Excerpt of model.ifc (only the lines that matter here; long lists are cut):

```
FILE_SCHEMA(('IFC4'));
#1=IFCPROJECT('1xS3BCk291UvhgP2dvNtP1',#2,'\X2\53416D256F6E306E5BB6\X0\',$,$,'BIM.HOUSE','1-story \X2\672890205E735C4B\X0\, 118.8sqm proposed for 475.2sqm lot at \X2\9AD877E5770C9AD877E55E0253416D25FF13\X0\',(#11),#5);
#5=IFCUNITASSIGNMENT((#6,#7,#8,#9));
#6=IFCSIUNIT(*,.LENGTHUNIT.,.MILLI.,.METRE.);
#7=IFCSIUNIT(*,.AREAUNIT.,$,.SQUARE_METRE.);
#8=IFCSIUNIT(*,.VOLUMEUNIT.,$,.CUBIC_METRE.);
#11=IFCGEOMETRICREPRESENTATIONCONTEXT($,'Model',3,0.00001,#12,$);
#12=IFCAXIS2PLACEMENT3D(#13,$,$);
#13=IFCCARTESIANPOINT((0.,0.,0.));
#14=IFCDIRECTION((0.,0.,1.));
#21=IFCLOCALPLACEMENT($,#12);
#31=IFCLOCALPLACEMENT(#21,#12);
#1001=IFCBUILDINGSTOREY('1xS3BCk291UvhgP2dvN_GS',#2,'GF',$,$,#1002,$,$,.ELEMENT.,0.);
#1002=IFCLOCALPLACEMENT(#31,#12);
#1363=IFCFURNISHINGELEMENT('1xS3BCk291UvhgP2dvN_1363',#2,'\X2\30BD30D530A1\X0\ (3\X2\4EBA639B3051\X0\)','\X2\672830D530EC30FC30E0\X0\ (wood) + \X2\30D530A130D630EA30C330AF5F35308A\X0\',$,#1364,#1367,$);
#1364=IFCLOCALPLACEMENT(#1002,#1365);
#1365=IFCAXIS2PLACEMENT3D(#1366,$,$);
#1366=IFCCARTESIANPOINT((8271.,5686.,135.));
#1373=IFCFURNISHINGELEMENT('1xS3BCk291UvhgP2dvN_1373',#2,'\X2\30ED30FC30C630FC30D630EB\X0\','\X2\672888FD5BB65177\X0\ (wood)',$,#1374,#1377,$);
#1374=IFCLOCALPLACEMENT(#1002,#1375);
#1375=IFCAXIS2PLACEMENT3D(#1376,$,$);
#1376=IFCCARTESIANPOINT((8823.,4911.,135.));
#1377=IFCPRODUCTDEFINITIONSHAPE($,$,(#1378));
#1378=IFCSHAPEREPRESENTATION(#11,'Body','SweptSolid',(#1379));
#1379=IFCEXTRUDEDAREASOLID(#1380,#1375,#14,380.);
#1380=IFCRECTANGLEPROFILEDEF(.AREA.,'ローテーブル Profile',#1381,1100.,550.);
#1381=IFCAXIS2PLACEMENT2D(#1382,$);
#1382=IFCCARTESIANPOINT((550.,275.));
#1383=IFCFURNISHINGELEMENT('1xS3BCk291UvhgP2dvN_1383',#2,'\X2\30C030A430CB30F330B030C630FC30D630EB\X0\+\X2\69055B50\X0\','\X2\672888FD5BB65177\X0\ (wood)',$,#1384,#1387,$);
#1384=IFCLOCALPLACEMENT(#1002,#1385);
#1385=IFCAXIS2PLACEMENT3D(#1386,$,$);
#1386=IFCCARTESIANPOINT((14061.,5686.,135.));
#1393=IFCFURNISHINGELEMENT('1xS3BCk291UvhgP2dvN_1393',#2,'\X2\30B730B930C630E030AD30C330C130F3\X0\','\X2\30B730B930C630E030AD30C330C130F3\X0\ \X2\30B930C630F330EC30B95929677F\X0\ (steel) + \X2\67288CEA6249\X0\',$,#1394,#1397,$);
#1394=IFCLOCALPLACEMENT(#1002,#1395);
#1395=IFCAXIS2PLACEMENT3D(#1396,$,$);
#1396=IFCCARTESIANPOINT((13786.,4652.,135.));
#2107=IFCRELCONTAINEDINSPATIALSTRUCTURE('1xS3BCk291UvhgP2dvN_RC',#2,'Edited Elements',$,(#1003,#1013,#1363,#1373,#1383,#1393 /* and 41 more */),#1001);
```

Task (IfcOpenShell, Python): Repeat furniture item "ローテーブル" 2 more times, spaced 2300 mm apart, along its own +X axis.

```python
import ifcopenshell
import ifcopenshell.api.geometry
import ifcopenshell.api.root
import ifcopenshell.util.element
import ifcopenshell.util.placement

model = ifcopenshell.open("model.ifc")


def reuse_history(source, copy):
    """copy_class also copies each property set's owner history, people and application; keep the originals."""
    for rel in copy.IsDefinedBy:
        if rel.is_a("IfcRelDefinesByProperties") and (history := rel.RelatingPropertyDefinition.OwnerHistory):
            rel.RelatingPropertyDefinition.OwnerHistory = source.OwnerHistory
            ifcopenshell.util.element.remove_deep2(model, history)


source = model.by_id(1373)
base = ifcopenshell.util.placement.get_local_placement(source.ObjectPlacement)
step = base[:3, 0] * 2300.0

for i in range(1, 3):
    copy = ifcopenshell.api.root.copy_class(model, product=source)
    copy.Representation = ifcopenshell.util.element.copy_deep(
        model, source.Representation, exclude=["IfcGeometricRepresentationContext", "IfcRepresentationMap"]
    )
    reuse_history(source, copy)
    matrix = base.copy()
    matrix[:3, 3] += i * step
    print("added at", matrix[:3, 3].round(3) + 0.0)
    ifcopenshell.api.geometry.edit_object_placement(model, product=copy, matrix=matrix, is_si=False)

model.write("model_edited.ifc")
```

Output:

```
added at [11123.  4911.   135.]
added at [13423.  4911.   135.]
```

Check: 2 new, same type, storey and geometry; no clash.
